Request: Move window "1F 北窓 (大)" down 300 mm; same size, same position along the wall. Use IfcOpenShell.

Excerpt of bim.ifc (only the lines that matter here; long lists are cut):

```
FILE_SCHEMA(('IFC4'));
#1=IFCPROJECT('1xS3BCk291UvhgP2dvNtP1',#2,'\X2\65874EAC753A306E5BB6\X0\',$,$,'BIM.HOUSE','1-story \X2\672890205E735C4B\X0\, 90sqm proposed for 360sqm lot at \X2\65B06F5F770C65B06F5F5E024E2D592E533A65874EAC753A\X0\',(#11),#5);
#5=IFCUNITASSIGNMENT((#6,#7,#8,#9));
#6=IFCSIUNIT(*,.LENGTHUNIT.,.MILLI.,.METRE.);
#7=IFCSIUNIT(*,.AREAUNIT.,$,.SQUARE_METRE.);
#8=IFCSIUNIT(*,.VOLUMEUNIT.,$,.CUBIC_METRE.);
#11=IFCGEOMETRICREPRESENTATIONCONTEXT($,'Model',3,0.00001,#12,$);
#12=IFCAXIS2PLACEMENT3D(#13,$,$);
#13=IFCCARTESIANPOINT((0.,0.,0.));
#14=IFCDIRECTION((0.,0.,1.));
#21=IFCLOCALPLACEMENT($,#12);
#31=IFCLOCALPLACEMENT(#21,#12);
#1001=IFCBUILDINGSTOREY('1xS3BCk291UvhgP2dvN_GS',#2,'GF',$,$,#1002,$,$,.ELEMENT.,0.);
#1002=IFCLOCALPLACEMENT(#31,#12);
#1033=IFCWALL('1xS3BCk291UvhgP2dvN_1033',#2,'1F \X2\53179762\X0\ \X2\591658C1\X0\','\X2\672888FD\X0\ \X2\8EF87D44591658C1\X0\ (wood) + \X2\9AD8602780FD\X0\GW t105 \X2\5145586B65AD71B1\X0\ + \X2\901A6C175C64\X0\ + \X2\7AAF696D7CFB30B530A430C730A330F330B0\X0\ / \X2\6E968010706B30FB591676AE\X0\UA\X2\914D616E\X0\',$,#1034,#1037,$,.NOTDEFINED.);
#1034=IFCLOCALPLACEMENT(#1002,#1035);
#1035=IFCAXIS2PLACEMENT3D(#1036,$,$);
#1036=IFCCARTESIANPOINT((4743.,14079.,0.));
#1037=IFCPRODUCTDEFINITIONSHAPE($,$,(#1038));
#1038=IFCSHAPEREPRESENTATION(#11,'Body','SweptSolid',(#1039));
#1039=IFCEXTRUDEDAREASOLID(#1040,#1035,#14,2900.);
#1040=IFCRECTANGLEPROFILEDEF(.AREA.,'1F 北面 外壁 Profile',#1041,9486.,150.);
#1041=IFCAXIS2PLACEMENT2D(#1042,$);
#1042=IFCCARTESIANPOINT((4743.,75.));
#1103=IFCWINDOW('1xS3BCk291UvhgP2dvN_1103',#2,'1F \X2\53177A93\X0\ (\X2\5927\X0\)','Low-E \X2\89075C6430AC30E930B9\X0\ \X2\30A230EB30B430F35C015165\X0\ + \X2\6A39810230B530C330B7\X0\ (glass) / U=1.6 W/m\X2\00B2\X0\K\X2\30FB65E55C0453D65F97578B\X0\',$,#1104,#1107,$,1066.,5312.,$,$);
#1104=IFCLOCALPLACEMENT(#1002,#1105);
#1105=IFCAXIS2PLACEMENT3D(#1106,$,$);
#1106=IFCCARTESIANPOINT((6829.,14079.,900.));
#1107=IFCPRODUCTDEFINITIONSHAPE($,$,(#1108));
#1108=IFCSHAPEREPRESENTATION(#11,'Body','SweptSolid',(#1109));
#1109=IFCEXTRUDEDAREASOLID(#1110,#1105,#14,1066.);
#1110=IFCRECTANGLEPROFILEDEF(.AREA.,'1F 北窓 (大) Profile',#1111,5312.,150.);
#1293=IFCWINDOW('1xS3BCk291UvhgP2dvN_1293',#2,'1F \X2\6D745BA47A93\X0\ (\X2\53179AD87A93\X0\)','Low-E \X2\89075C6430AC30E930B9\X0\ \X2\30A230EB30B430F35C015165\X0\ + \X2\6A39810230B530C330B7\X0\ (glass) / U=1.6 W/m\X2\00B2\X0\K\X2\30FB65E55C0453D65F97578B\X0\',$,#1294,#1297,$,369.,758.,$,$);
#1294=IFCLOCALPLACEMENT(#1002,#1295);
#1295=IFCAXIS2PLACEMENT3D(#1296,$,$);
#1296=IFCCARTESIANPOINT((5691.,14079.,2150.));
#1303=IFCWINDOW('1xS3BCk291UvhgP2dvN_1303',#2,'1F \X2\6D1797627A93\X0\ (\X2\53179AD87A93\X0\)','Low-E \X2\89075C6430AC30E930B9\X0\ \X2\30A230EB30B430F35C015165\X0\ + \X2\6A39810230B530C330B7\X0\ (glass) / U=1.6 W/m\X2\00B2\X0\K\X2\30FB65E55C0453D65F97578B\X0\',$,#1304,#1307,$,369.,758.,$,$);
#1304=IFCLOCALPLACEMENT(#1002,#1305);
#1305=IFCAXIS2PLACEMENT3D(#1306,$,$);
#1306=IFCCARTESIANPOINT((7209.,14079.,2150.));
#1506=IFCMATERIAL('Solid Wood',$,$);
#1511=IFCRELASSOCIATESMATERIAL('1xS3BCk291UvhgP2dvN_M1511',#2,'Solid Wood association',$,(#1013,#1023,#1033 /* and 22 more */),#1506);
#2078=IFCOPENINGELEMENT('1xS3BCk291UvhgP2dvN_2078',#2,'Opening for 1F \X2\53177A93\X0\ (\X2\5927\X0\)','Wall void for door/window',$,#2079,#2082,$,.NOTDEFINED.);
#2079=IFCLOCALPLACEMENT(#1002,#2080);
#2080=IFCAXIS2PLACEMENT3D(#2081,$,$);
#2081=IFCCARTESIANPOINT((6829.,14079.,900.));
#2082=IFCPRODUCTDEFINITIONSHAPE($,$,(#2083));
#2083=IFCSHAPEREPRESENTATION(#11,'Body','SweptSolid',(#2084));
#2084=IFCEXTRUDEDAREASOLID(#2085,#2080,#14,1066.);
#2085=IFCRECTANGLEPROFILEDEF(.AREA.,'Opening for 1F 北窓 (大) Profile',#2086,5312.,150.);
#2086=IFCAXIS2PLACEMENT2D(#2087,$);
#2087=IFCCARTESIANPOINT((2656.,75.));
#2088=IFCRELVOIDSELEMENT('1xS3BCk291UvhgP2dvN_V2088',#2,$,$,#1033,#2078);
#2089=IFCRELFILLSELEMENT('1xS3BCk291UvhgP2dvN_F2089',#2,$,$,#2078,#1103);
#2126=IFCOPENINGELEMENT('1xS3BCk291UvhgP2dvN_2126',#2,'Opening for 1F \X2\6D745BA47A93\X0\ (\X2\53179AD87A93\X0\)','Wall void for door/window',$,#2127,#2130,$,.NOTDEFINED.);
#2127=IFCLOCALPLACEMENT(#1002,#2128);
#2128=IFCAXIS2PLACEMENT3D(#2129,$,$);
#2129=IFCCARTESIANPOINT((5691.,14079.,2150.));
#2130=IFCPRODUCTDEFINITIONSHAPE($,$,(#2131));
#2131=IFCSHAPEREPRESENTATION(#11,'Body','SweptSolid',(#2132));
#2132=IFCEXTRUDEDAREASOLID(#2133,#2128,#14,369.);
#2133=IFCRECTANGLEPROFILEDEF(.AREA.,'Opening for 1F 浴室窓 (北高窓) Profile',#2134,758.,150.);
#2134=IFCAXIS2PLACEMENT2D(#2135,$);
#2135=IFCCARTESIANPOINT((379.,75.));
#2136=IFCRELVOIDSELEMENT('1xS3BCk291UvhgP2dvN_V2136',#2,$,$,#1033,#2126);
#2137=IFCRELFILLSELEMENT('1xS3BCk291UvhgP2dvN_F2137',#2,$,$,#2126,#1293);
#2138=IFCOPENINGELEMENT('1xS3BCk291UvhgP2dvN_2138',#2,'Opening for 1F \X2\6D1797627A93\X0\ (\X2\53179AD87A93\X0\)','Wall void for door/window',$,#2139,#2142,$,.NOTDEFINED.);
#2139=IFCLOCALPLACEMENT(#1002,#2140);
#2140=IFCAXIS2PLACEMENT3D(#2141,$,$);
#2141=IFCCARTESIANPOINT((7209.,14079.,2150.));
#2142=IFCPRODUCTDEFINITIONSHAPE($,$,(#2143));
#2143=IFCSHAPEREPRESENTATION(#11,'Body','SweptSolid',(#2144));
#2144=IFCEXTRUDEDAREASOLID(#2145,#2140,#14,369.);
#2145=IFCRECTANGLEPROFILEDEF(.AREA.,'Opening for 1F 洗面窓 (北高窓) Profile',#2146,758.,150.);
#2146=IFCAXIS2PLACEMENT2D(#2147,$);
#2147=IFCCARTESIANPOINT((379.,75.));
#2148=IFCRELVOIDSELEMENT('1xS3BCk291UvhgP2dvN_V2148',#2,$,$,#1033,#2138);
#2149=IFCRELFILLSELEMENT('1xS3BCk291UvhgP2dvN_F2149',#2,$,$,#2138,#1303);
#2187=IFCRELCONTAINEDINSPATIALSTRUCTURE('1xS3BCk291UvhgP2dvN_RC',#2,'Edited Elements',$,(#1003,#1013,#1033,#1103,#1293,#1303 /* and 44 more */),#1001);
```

```python
import numpy as np
import ifcopenshell
import ifcopenshell.api.geometry
import ifcopenshell.util.placement
import ifcopenshell.util.unit

model = ifcopenshell.open("bim.ifc")
unit_scale = ifcopenshell.util.unit.calculate_unit_scale(model)

window = model.by_id(1103)
opening = window.FillsVoids[0].RelatingOpeningElement
dz = -300.0

shift = np.array([0.0, 0.0, dz])
# The window is not placed relative to its opening, so move both.
for product in (opening, window):
    matrix = ifcopenshell.util.placement.get_local_placement(product.ObjectPlacement)
    matrix[:3, 3] += shift
    ifcopenshell.api.geometry.edit_object_placement(model, product=product, matrix=matrix, is_si=False)

print(f"moved by {dz * unit_scale:+.3f} m")

model.write("bim_edited.ifc")
```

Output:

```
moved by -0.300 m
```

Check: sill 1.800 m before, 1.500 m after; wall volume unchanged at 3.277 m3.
